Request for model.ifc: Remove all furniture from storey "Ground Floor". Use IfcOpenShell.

First a look at what the model holds.

```python
import ifcopenshell
import ifcopenshell.util.element

model = ifcopenshell.open("model.ifc")
print(model.schema)
storey = next(s for s in model.by_type("IfcBuildingStorey") if s.Name == "Ground Floor")
furniture = [e for e in ifcopenshell.util.element.get_decomposition(storey) if e.is_a("IfcFurnishingElement")]
seen = {}
for e in furniture:
    element_type = ifcopenshell.util.element.get_type(e)
    name = element_type.Name if element_type not in (None, e) else None
    seen[name] = seen.get(name, 0) + 1
for name, count in sorted(seen.items(), key=str):
    print(count, "x", name)
```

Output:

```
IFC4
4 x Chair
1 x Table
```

```python
import ifcopenshell
import ifcopenshell.api.root
import ifcopenshell.util.element

model = ifcopenshell.open("model.ifc")

storey = next(s for s in model.by_type("IfcBuildingStorey") if s.Name == "Ground Floor")
furniture = [e for e in ifcopenshell.util.element.get_decomposition(storey) if e.is_a("IfcFurnishingElement")]

for e in furniture:
    ifcopenshell.api.root.remove_product(model, product=e)
print(len(furniture), "removed")

model.write("model_updated.ifc")
```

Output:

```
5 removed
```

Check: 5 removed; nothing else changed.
